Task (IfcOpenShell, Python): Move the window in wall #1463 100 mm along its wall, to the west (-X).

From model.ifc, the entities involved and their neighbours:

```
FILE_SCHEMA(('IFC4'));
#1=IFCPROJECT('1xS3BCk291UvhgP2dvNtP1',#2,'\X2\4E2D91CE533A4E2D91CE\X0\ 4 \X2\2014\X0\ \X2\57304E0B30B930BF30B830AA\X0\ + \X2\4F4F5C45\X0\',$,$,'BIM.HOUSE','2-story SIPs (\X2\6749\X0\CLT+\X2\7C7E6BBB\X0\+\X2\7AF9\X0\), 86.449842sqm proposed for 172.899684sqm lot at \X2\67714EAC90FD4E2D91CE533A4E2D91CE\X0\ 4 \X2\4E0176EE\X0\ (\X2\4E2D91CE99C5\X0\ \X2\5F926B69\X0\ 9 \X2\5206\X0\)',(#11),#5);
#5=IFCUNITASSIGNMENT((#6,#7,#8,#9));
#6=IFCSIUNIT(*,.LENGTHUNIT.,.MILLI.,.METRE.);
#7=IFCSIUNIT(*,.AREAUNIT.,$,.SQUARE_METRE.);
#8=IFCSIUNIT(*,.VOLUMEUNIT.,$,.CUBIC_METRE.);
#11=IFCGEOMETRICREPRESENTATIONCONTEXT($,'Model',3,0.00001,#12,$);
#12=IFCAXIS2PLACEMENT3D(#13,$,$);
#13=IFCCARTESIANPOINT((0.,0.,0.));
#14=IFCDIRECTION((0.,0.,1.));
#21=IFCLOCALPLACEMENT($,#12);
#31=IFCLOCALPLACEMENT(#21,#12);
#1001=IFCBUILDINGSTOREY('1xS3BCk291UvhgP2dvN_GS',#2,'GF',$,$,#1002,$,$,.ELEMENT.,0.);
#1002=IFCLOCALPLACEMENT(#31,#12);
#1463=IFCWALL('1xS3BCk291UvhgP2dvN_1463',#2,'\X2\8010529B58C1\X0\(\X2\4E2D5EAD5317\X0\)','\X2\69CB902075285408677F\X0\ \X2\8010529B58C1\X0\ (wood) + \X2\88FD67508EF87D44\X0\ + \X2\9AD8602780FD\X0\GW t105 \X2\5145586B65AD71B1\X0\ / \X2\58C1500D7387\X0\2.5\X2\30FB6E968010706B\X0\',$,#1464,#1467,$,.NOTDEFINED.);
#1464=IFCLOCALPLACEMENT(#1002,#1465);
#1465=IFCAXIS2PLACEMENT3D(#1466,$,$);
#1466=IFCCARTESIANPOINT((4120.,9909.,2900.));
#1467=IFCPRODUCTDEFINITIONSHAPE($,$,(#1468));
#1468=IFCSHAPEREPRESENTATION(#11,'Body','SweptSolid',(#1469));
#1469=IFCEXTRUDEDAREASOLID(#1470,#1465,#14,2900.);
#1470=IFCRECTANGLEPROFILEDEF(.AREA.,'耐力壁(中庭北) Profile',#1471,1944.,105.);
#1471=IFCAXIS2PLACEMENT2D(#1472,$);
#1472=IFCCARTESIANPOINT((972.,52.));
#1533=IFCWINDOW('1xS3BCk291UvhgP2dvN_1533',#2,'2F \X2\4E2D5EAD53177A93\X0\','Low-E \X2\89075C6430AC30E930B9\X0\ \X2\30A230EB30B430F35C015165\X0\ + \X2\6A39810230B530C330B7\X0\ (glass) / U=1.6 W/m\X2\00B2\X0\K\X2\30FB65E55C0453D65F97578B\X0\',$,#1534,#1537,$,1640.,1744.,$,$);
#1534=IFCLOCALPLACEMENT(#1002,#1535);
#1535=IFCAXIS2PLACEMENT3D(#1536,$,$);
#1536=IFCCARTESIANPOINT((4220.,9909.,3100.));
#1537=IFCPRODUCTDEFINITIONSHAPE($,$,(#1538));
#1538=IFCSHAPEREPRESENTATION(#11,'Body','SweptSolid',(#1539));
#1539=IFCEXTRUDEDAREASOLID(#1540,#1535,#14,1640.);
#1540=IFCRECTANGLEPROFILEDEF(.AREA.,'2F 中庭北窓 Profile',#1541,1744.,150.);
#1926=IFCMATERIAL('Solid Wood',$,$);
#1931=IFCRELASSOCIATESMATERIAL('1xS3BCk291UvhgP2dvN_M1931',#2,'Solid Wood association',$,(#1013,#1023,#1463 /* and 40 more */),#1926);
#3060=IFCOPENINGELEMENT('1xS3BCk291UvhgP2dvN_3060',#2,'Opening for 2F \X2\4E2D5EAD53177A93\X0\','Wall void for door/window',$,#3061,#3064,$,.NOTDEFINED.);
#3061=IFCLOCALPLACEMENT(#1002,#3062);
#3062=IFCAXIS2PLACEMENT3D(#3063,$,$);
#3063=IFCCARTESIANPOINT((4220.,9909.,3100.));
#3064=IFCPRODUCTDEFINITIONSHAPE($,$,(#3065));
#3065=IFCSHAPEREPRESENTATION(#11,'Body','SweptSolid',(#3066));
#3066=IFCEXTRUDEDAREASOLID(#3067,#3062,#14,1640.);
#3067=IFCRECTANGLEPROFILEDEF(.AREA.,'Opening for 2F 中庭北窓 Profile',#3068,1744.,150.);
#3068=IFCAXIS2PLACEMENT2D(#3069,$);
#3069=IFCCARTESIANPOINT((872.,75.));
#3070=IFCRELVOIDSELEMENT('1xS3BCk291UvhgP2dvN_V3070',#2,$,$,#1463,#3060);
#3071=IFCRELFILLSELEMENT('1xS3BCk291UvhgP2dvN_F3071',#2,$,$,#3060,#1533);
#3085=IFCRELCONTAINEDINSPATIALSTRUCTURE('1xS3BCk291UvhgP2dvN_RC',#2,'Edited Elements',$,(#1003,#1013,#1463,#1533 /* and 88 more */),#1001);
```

```python
import ifcopenshell
import ifcopenshell.api.geometry
import ifcopenshell.util.placement

model = ifcopenshell.open("model.ifc")

window = model.by_guid("1xS3BCk291UvhgP2dvN_1533")
opening = window.FillsVoids[0].RelatingOpeningElement
wall = opening.VoidsElements[0].RelatingBuildingElement

wall_matrix = ifcopenshell.util.placement.get_local_placement(wall.ObjectPlacement)
shift = wall_matrix[:3, 0] * -100.0
before = ifcopenshell.util.placement.get_local_placement(window.ObjectPlacement)[:3, 3].copy()

# The window is not placed relative to its opening, so move both.
for product in (opening, window):
    matrix = ifcopenshell.util.placement.get_local_placement(product.ObjectPlacement)
    matrix[:3, 3] += shift
    ifcopenshell.api.geometry.edit_object_placement(model, product=product, matrix=matrix, is_si=False)

after = ifcopenshell.util.placement.get_local_placement(window.ObjectPlacement)[:3, 3]
print("window moved by", (after - before).round(3) + 0.0)

model.write("model_rev.ifc")
```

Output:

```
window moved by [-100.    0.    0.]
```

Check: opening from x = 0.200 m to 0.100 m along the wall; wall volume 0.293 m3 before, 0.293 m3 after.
